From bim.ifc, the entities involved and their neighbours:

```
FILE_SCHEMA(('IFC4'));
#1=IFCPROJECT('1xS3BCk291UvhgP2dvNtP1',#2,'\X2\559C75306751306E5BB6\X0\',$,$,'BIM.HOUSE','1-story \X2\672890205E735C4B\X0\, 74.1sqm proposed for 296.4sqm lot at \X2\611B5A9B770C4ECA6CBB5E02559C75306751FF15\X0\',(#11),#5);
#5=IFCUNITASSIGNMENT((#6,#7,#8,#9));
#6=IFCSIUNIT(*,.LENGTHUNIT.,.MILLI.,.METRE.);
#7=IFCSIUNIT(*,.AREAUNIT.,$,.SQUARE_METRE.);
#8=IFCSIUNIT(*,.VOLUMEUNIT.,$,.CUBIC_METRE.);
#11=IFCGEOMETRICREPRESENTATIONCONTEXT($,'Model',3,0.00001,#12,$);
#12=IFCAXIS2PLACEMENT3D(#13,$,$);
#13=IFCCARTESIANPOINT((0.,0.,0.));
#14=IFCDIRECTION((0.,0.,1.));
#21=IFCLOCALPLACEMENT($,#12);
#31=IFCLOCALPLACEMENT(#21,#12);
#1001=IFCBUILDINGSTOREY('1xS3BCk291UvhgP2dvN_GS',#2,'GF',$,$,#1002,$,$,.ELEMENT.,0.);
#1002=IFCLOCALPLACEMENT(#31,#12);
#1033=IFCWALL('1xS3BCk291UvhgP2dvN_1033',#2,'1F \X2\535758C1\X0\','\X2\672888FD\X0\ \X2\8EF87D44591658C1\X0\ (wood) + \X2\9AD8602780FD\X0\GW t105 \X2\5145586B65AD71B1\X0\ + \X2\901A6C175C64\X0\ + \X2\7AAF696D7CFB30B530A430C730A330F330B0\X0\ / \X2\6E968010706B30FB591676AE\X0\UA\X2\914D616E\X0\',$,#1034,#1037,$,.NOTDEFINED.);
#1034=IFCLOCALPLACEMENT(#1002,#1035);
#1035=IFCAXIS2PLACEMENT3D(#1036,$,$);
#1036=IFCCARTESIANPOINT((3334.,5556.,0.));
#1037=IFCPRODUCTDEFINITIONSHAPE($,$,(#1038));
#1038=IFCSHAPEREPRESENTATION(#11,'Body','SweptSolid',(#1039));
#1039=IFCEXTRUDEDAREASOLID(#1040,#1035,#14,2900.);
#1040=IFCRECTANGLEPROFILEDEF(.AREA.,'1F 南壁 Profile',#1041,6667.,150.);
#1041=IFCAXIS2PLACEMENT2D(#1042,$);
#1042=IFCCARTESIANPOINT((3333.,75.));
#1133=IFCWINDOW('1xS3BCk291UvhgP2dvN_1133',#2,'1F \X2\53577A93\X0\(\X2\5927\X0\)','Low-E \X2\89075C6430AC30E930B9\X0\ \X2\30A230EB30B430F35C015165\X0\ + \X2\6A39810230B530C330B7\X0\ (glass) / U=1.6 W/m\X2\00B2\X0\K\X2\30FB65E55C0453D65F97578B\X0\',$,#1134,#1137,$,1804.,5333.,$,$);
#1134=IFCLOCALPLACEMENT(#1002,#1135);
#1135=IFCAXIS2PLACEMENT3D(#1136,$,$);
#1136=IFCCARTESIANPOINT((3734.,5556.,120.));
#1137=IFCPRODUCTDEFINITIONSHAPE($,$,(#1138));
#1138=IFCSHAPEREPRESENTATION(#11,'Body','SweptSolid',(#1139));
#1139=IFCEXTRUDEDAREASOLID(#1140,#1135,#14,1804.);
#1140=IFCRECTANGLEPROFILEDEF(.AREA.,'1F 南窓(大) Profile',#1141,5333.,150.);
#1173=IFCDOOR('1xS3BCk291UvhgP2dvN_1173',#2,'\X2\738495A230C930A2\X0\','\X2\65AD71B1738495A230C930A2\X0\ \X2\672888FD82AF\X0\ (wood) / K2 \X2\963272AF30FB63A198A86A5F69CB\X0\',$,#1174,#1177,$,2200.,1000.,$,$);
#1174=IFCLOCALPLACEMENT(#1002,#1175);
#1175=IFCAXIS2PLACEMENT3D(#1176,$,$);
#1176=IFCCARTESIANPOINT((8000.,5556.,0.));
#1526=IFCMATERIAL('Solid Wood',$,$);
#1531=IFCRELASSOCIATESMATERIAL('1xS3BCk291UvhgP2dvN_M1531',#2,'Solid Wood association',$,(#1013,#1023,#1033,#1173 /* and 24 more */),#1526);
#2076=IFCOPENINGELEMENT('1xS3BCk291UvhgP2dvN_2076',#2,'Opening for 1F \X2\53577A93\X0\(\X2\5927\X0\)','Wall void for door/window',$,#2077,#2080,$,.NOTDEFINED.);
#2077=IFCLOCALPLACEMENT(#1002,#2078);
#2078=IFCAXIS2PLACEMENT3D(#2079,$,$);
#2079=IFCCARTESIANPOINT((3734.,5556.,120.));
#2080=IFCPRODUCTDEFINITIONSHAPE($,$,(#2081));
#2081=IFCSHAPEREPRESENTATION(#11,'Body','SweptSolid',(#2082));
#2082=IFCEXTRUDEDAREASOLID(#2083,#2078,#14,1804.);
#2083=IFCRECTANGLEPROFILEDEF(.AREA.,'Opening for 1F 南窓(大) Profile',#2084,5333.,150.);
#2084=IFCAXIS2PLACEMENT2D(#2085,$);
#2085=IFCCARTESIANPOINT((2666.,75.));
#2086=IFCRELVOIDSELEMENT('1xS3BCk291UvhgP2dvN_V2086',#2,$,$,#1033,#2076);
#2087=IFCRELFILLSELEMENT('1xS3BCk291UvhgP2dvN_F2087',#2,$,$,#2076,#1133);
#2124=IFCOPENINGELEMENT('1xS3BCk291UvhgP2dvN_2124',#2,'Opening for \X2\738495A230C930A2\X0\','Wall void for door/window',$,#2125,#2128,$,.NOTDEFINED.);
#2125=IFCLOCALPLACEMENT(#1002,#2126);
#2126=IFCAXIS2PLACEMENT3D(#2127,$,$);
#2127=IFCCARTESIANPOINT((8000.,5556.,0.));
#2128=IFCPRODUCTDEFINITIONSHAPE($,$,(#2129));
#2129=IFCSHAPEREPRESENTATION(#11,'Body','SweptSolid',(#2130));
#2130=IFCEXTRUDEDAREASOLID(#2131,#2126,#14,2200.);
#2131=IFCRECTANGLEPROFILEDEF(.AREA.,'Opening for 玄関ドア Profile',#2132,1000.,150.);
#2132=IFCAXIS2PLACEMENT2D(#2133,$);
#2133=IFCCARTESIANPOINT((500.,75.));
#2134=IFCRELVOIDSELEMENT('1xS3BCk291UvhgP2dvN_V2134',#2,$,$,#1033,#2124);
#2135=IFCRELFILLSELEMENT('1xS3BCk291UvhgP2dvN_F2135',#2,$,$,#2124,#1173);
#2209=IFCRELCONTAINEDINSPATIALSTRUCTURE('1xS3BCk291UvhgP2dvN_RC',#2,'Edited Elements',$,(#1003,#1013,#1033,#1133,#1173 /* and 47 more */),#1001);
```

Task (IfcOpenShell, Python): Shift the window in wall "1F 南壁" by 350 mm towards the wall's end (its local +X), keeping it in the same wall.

```python
import ifcopenshell
import ifcopenshell.api.geometry
import ifcopenshell.util.placement
import ifcopenshell.util.unit

model = ifcopenshell.open("bim.ifc")
unit_scale = ifcopenshell.util.unit.calculate_unit_scale(model)

window = model.by_guid("1xS3BCk291UvhgP2dvN_1133")
opening = window.FillsVoids[0].RelatingOpeningElement
wall = opening.VoidsElements[0].RelatingBuildingElement

wall_matrix = ifcopenshell.util.placement.get_local_placement(wall.ObjectPlacement)
shift = wall_matrix[:3, 0] * 0.35 / unit_scale
before = ifcopenshell.util.placement.get_local_placement(window.ObjectPlacement)[:3, 3].copy()

# The window is not placed relative to its opening, so move both.
for product in (opening, window):
    matrix = ifcopenshell.util.placement.get_local_placement(product.ObjectPlacement)
    matrix[:3, 3] += shift
    ifcopenshell.api.geometry.edit_object_placement(model, product=product, matrix=matrix, is_si=False)

after = ifcopenshell.util.placement.get_local_placement(window.ObjectPlacement)[:3, 3]
print("window moved by", (after - before).round(3) + 0.0)

model.write("bim_v2.ifc")
```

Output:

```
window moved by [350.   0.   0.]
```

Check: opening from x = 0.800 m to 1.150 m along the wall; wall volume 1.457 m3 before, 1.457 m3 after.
